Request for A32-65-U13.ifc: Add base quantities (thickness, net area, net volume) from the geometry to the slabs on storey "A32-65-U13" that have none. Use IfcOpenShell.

First a look at what the model holds.

```python
import ifcopenshell
import ifcopenshell.util.element
import ifcopenshell.util.unit

model = ifcopenshell.open("A32-65-U13.ifc")
print(model.schema)
for unit_type in ("LENGTHUNIT", "AREAUNIT", "VOLUMEUNIT"):
    print(unit_type, ifcopenshell.util.unit.calculate_unit_scale(model, unit_type))
storey = next(s for s in model.by_type("IfcBuildingStorey") if s.Name == "A32-65-U13")
slabs = [e for e in ifcopenshell.util.element.get_decomposition(storey) if e.is_a("IfcSlab")]
for e in sorted(slabs, key=lambda e: e.id()):
    print(e.id(), e.is_a(), e.Name, list(ifcopenshell.util.element.get_psets(e, qtos_only=True)), sep=" | ")
```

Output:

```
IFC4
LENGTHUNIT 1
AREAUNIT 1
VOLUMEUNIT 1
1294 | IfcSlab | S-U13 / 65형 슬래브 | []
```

```python
import ifcopenshell
import ifcopenshell.api.pset
import ifcopenshell.geom
import ifcopenshell.util.element
import ifcopenshell.util.shape
import ifcopenshell.util.unit

model = ifcopenshell.open("A32-65-U13.ifc")
unit_scale = ifcopenshell.util.unit.calculate_unit_scale(model)
area_scale = ifcopenshell.util.unit.calculate_unit_scale(model, "AREAUNIT")
volume_scale = ifcopenshell.util.unit.calculate_unit_scale(model, "VOLUMEUNIT")
settings = ifcopenshell.geom.settings()

storey = next(s for s in model.by_type("IfcBuildingStorey") if s.Name == "A32-65-U13")
slabs = [e for e in ifcopenshell.util.element.get_decomposition(storey) if e.is_a("IfcSlab")]

for e in sorted(slabs, key=lambda e: e.id()):
    if ifcopenshell.util.element.get_psets(e, qtos_only=True, should_inherit=False):
        continue
    # Geometry comes back in metres, in the element's own axes.
    shape = ifcopenshell.geom.create_shape(settings, e)
    values = {
        "Width": ifcopenshell.util.shape.get_z(shape.geometry) / unit_scale,
        "NetArea": ifcopenshell.util.shape.get_footprint_area(shape.geometry) / area_scale,
        "NetVolume": ifcopenshell.util.shape.get_volume(shape.geometry) / volume_scale,
    }
    qto = ifcopenshell.api.pset.add_qto(model, product=e, name="Qto_SlabBaseQuantities")
    ifcopenshell.api.pset.edit_qto(model, qto=qto, properties=values)
    print(e.id(), {k: round(v, 3) for k, v in values.items()})

model.write("A32-65-U13_v2.ifc")
```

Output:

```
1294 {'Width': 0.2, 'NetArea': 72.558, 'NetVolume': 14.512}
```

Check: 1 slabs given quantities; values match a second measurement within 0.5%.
